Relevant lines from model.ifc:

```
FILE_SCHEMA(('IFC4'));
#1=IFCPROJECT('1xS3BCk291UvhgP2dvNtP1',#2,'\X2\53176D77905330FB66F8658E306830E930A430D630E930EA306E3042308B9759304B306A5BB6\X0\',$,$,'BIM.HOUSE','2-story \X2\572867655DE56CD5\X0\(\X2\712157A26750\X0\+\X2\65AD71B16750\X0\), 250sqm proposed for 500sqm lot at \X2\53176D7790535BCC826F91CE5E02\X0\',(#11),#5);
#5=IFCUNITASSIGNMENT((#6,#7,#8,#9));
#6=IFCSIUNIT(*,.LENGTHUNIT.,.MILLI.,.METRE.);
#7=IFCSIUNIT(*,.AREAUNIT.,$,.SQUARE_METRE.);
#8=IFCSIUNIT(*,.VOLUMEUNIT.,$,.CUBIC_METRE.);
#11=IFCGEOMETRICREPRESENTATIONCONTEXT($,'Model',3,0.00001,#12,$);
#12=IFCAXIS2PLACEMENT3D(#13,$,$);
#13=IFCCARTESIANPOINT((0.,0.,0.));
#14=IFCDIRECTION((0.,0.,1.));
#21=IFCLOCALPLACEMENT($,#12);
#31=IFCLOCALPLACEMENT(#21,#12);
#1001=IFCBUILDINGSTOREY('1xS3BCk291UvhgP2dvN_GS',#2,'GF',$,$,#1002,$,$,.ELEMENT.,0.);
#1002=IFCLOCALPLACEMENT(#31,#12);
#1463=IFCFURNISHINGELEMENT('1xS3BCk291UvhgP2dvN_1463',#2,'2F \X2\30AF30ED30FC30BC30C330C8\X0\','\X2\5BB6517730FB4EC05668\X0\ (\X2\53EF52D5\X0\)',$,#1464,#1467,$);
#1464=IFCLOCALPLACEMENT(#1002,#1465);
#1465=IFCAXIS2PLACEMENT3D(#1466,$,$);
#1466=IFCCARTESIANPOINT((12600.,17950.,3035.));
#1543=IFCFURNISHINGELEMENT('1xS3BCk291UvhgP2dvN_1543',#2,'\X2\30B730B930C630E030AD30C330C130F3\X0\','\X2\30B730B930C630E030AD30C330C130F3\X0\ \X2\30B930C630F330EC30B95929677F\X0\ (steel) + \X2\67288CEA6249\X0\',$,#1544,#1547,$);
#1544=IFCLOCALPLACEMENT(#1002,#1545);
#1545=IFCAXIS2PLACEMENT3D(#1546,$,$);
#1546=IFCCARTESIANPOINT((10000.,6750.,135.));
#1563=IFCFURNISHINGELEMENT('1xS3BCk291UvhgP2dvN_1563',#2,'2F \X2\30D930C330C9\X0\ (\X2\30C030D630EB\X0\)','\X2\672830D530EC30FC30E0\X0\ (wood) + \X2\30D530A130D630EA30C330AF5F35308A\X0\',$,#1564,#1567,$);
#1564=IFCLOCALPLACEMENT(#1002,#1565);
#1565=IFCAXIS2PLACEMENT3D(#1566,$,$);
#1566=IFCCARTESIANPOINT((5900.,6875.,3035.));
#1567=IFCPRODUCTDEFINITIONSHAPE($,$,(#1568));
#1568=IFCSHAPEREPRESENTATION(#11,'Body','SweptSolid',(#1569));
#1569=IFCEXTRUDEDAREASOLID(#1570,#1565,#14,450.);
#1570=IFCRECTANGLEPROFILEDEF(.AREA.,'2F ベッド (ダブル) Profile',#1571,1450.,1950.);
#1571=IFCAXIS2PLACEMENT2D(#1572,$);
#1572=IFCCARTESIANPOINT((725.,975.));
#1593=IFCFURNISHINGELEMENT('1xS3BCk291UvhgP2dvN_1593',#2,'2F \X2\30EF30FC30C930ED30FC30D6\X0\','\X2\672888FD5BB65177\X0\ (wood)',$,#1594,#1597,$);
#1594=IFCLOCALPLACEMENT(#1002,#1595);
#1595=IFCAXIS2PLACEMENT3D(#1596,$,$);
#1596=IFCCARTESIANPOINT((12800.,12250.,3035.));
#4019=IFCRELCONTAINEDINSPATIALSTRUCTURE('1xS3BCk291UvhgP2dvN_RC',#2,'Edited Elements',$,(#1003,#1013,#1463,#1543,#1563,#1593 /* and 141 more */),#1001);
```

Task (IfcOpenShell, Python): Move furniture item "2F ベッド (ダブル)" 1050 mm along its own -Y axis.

```python
import ifcopenshell
import ifcopenshell.api.geometry
import ifcopenshell.util.placement

model = ifcopenshell.open("model.ifc")

item = model.by_id(1563)
matrix = ifcopenshell.util.placement.get_local_placement(item.ObjectPlacement)
matrix[:3, 3] -= matrix[:3, 1] * 1050.0
ifcopenshell.api.geometry.edit_object_placement(model, product=item, matrix=matrix, is_si=False)

print(ifcopenshell.util.placement.get_local_placement(item.ObjectPlacement).round(3) + 0.0)

model.write("model_v2.ifc")
```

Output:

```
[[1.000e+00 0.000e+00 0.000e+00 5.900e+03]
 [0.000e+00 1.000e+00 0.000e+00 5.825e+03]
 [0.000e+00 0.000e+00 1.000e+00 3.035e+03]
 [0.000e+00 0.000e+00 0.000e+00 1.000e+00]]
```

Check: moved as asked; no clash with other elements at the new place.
